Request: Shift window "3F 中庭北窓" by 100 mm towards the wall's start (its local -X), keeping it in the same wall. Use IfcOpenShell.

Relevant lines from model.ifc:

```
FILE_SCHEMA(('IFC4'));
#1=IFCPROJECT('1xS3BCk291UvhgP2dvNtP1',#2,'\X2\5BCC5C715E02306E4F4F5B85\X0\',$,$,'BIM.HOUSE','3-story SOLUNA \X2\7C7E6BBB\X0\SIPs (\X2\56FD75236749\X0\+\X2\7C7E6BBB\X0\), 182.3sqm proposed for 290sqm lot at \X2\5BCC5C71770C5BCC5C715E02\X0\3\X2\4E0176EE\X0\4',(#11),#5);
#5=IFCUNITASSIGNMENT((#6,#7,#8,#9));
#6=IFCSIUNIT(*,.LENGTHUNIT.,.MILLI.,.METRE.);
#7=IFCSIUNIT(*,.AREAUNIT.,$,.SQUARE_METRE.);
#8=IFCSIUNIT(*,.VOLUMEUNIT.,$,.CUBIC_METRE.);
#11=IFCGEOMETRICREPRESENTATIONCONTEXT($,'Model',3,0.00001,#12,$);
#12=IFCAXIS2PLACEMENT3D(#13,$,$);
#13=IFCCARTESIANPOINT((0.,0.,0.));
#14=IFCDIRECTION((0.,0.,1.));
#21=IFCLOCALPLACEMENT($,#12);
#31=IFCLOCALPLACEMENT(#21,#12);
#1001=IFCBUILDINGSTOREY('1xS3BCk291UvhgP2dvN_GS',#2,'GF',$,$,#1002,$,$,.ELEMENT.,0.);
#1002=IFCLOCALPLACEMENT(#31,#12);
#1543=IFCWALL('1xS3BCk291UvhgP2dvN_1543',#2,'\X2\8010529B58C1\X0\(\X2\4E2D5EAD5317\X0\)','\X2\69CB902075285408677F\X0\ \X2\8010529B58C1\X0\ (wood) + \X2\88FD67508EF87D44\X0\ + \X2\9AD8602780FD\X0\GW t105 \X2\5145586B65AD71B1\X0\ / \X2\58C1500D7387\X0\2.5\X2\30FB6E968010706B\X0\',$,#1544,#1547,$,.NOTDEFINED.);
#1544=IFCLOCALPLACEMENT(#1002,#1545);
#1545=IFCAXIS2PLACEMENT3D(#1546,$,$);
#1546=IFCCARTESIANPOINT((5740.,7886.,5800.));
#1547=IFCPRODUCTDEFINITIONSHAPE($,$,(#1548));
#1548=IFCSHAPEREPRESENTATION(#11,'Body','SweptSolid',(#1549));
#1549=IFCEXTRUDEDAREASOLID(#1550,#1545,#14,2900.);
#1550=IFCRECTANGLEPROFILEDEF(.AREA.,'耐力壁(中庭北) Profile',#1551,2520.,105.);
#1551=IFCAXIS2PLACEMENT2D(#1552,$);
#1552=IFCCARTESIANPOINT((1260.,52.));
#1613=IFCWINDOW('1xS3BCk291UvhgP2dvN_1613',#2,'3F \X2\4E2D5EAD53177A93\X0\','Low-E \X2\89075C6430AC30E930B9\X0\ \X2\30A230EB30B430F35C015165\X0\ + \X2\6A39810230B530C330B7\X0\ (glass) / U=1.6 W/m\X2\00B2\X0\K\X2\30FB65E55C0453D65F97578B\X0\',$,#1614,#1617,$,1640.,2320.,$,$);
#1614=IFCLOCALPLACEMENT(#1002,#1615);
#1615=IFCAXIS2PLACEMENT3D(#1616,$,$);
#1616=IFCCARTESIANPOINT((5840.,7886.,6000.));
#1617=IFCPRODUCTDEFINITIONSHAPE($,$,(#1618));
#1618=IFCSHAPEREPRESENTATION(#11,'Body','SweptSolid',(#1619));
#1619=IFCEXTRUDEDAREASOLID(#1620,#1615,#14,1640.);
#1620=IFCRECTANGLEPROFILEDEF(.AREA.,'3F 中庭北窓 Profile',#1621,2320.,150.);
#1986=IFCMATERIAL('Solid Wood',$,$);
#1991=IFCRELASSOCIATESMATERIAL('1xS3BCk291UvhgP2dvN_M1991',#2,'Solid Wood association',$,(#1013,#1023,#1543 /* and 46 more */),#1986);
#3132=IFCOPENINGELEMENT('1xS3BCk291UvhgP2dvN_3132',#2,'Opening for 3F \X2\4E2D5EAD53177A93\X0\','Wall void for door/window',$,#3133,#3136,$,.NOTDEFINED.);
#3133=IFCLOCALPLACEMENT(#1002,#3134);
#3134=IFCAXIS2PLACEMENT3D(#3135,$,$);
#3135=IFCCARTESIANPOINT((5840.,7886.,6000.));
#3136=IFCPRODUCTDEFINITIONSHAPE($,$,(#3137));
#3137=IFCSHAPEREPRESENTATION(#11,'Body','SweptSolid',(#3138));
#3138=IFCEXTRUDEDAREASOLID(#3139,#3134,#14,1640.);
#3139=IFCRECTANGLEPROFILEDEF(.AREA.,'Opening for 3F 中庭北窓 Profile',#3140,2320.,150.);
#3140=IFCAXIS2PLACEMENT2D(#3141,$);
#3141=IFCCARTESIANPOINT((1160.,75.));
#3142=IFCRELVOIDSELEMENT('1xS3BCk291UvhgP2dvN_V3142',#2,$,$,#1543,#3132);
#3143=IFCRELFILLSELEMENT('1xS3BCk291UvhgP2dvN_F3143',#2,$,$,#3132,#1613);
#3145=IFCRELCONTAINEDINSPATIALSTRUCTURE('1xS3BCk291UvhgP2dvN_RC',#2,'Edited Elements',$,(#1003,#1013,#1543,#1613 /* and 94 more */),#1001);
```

```python
import ifcopenshell
import ifcopenshell.api.geometry
import ifcopenshell.util.placement

model = ifcopenshell.open("model.ifc")

window = model.by_guid("1xS3BCk291UvhgP2dvN_1613")
opening = window.FillsVoids[0].RelatingOpeningElement
wall = opening.VoidsElements[0].RelatingBuildingElement

wall_matrix = ifcopenshell.util.placement.get_local_placement(wall.ObjectPlacement)
shift = wall_matrix[:3, 0] * -100.0
before = ifcopenshell.util.placement.get_local_placement(window.ObjectPlacement)[:3, 3].copy()

# The window is not placed relative to its opening, so move both.
for product in (opening, window):
    matrix = ifcopenshell.util.placement.get_local_placement(product.ObjectPlacement)
    matrix[:3, 3] += shift
    ifcopenshell.api.geometry.edit_object_placement(model, product=product, matrix=matrix, is_si=False)

after = ifcopenshell.util.placement.get_local_placement(window.ObjectPlacement)[:3, 3]
print("window moved by", (after - before).round(3) + 0.0)

model.write("model_edited.ifc")
```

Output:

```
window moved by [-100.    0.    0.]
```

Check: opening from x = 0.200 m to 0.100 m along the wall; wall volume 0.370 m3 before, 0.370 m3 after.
